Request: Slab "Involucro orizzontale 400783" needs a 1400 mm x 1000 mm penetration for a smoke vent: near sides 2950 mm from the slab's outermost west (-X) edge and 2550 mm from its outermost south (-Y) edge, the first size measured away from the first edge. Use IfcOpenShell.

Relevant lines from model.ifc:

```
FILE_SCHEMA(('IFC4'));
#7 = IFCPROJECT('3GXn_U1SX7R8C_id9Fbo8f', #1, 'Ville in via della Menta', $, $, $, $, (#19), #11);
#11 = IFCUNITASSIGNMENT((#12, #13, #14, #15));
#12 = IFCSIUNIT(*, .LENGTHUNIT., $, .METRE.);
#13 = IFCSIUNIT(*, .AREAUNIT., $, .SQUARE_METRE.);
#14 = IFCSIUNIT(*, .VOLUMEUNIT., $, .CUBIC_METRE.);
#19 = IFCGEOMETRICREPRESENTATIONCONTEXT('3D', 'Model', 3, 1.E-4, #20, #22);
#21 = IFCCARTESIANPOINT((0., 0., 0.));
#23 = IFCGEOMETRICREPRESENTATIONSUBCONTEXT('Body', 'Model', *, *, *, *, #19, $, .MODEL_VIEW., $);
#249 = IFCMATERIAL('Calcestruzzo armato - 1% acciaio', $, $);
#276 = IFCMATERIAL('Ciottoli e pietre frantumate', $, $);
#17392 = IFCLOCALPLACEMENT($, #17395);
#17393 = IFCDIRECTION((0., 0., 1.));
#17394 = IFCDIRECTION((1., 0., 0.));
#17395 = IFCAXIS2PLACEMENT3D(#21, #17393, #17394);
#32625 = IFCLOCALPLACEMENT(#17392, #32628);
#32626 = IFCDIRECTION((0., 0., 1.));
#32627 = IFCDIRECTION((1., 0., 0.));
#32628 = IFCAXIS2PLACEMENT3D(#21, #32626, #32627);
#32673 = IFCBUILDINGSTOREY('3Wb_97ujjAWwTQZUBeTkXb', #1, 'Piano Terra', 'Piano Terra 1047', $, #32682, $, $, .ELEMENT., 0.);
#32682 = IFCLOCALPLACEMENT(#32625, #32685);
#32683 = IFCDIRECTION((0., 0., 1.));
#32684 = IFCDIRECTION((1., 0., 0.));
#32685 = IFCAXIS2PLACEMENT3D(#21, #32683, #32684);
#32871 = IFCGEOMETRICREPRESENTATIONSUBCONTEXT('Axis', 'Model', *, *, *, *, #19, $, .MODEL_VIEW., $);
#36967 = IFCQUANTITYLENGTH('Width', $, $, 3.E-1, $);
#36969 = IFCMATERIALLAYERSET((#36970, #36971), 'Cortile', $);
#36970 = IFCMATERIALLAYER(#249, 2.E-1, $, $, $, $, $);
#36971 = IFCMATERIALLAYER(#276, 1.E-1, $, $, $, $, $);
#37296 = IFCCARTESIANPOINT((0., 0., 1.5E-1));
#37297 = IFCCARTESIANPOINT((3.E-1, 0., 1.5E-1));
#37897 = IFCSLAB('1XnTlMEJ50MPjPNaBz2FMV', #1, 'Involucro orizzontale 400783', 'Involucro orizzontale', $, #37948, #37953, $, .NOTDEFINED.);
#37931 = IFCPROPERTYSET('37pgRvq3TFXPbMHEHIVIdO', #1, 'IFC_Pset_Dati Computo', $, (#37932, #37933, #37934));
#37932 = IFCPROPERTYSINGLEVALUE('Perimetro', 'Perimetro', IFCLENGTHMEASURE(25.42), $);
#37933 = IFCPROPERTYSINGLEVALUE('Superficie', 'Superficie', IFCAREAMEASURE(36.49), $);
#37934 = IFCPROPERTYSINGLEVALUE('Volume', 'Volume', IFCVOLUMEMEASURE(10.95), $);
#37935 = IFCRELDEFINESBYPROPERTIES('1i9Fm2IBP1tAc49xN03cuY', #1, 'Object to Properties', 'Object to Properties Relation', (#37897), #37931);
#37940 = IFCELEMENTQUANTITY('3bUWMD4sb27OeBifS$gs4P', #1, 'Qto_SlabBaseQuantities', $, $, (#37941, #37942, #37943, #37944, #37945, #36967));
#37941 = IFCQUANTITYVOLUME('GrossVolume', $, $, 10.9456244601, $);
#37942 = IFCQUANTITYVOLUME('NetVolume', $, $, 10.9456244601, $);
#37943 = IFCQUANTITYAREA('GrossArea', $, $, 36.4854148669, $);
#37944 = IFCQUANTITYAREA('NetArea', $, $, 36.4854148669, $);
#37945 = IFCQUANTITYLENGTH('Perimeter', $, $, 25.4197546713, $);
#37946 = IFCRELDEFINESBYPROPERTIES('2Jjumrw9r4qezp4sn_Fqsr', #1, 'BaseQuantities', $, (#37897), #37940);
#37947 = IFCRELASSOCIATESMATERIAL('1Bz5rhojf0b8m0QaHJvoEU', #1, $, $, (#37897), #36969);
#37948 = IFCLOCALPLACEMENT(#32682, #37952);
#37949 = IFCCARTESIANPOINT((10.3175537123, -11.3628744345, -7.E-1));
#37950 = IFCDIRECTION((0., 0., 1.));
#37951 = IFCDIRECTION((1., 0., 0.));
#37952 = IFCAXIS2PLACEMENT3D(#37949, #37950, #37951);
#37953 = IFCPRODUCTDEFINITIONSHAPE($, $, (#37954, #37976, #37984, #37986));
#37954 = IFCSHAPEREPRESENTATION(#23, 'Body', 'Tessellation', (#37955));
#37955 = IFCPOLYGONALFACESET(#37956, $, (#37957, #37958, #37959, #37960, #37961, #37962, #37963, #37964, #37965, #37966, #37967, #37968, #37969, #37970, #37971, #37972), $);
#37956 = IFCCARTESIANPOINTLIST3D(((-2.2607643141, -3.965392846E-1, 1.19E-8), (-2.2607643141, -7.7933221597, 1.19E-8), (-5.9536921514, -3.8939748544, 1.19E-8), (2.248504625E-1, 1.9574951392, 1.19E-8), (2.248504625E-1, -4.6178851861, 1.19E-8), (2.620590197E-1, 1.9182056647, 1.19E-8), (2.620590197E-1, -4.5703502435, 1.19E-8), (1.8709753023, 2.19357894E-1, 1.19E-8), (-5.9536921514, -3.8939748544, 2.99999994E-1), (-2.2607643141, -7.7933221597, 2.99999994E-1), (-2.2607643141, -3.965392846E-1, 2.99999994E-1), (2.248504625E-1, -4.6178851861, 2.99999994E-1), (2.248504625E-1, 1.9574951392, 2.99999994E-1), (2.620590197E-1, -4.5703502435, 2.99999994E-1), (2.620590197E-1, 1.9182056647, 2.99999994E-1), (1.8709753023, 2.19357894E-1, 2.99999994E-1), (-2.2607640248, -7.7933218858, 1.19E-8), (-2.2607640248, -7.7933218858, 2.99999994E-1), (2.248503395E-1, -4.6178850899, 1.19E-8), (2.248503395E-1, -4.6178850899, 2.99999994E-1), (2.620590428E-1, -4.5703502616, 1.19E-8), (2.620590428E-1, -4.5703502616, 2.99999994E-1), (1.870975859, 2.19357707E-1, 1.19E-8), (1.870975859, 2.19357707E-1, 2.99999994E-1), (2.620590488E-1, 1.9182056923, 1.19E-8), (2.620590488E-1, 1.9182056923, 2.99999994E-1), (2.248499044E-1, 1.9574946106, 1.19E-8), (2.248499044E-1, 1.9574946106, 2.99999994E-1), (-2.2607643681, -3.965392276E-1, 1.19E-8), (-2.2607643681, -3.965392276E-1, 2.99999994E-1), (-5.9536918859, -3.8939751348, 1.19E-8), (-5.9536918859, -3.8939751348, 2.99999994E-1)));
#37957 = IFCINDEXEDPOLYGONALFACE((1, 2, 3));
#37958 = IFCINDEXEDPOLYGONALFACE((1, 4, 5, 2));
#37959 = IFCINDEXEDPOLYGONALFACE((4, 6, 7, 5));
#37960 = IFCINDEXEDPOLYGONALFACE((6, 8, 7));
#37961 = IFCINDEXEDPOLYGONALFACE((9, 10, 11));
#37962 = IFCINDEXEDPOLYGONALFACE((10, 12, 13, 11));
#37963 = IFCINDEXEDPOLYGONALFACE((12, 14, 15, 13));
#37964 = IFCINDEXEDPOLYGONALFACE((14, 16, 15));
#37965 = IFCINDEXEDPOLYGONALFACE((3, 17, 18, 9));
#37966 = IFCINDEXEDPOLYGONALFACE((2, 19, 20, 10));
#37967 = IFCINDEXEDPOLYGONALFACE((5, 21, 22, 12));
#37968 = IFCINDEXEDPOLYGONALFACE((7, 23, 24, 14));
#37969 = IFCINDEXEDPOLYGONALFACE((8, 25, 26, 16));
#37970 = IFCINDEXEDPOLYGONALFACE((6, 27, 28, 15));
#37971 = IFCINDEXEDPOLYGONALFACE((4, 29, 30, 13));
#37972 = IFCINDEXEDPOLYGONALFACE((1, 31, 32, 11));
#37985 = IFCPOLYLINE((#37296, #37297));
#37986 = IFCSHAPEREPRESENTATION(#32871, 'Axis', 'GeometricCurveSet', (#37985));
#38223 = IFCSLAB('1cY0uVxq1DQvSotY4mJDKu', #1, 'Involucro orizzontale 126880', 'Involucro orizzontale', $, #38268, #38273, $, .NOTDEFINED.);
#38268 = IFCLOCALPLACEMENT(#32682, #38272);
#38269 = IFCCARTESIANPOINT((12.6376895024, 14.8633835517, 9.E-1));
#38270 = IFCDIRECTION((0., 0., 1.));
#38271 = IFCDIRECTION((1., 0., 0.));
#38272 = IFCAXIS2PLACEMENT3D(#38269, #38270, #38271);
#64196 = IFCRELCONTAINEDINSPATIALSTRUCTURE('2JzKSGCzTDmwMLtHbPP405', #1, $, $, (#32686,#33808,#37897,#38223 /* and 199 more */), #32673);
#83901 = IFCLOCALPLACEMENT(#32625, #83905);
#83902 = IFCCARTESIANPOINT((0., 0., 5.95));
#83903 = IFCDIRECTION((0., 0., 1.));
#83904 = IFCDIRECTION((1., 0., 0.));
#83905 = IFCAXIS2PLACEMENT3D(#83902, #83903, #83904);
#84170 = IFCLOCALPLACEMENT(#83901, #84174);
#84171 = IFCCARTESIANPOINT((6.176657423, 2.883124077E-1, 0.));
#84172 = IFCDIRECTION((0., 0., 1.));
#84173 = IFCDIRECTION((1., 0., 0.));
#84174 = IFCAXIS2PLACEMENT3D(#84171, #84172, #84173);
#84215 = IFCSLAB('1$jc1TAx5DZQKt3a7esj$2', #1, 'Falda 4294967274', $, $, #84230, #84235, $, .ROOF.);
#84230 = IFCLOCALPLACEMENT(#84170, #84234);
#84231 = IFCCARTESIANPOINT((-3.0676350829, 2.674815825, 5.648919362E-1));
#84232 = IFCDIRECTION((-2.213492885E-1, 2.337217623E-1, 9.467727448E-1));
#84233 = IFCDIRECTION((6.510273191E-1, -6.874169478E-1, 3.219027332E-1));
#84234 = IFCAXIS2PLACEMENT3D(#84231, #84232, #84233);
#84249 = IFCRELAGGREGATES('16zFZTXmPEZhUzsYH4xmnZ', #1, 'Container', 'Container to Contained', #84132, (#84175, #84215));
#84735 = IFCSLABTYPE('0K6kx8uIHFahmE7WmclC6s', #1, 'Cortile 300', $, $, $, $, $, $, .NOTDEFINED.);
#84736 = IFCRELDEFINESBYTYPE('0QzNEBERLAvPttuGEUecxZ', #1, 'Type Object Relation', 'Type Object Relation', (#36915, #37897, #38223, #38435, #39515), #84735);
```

```python
import numpy as np
import ifcopenshell
import ifcopenshell.api.feature
import ifcopenshell.api.geometry
import ifcopenshell.api.pset
import ifcopenshell.api.root
import ifcopenshell.geom
import ifcopenshell.util.element
import ifcopenshell.util.placement
import ifcopenshell.util.representation
import ifcopenshell.util.shape
import ifcopenshell.util.unit

model = ifcopenshell.open("model.ifc")
unit_scale = ifcopenshell.util.unit.calculate_unit_scale(model)
area_scale = ifcopenshell.util.unit.calculate_unit_scale(model, "AREAUNIT")
volume_scale = ifcopenshell.util.unit.calculate_unit_scale(model, "VOLUMEUNIT")
settings = ifcopenshell.geom.settings()


def volume(element):
    """Net volume in cubic metres, openings subtracted."""
    shape = ifcopenshell.geom.create_shape(settings, element)
    return ifcopenshell.util.shape.get_volume(shape.geometry)


slab = model.by_id(37897)
before = volume(slab)

# Extent in the slab's own axes, in metres. The edges named are its -X and -Y sides.
slab_shape = ifcopenshell.geom.create_shape(settings, slab)
vertices = ifcopenshell.util.shape.get_vertices(slab_shape.geometry)
x_min, y_min, bottom = vertices.min(axis=0)
top = vertices[:, 2].max()

opening = ifcopenshell.api.root.create_entity(model, ifc_class="IfcOpeningElement", name="Smoke vent opening", predefined_type="OPENING")
context = ifcopenshell.util.representation.get_context(model, "Model", "Body", "MODEL_VIEW")
width, depth = 1.4, 1
outline = [(0.0, 0.0), (width, 0.0), (width, depth), (0.0, depth), (0.0, 0.0)]
# Overshoot both faces by 50 mm so the cut is clean.
shape = ifcopenshell.api.geometry.add_slab_representation(
    model, context=context, depth=top - bottom + 0.1, polyline=outline
)
ifcopenshell.api.geometry.assign_representation(model, product=opening, representation=shape)

matrix = ifcopenshell.util.placement.get_local_placement(slab.ObjectPlacement)
matrix[:, 3] = matrix @ np.append(np.array([x_min + 2.95, y_min + 2.55, bottom - 0.05]) / unit_scale, 1.0)
ifcopenshell.api.geometry.edit_object_placement(model, product=opening, matrix=matrix, is_si=False)
ifcopenshell.api.feature.add_feature(model, feature=opening, element=slab)

after = volume(slab)

# Update the slab's stored quantities.
pset = model.by_id(ifcopenshell.util.element.get_pset(slab, "IFC_Pset_Dati Computo", should_inherit=False)["id"])
ifcopenshell.api.pset.edit_pset(model, pset=pset, properties={
    "Superficie": model.create_entity("IfcAreaMeasure", after / (top - bottom) / area_scale),
    "Volume": model.create_entity("IfcVolumeMeasure", after / volume_scale),
})
qto = model.by_id(ifcopenshell.util.element.get_pset(slab, "Qto_SlabBaseQuantities", should_inherit=False)["id"])
ifcopenshell.api.pset.edit_qto(model, qto=qto, properties={
    "NetVolume": after / volume_scale,
    "NetArea": after / (top - bottom) / area_scale,
})

print(f"slab volume {before:.3f} -> {after:.3f} m3")

model.write("model_updated.ifc")
```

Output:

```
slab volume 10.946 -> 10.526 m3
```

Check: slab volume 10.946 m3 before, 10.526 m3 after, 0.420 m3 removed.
